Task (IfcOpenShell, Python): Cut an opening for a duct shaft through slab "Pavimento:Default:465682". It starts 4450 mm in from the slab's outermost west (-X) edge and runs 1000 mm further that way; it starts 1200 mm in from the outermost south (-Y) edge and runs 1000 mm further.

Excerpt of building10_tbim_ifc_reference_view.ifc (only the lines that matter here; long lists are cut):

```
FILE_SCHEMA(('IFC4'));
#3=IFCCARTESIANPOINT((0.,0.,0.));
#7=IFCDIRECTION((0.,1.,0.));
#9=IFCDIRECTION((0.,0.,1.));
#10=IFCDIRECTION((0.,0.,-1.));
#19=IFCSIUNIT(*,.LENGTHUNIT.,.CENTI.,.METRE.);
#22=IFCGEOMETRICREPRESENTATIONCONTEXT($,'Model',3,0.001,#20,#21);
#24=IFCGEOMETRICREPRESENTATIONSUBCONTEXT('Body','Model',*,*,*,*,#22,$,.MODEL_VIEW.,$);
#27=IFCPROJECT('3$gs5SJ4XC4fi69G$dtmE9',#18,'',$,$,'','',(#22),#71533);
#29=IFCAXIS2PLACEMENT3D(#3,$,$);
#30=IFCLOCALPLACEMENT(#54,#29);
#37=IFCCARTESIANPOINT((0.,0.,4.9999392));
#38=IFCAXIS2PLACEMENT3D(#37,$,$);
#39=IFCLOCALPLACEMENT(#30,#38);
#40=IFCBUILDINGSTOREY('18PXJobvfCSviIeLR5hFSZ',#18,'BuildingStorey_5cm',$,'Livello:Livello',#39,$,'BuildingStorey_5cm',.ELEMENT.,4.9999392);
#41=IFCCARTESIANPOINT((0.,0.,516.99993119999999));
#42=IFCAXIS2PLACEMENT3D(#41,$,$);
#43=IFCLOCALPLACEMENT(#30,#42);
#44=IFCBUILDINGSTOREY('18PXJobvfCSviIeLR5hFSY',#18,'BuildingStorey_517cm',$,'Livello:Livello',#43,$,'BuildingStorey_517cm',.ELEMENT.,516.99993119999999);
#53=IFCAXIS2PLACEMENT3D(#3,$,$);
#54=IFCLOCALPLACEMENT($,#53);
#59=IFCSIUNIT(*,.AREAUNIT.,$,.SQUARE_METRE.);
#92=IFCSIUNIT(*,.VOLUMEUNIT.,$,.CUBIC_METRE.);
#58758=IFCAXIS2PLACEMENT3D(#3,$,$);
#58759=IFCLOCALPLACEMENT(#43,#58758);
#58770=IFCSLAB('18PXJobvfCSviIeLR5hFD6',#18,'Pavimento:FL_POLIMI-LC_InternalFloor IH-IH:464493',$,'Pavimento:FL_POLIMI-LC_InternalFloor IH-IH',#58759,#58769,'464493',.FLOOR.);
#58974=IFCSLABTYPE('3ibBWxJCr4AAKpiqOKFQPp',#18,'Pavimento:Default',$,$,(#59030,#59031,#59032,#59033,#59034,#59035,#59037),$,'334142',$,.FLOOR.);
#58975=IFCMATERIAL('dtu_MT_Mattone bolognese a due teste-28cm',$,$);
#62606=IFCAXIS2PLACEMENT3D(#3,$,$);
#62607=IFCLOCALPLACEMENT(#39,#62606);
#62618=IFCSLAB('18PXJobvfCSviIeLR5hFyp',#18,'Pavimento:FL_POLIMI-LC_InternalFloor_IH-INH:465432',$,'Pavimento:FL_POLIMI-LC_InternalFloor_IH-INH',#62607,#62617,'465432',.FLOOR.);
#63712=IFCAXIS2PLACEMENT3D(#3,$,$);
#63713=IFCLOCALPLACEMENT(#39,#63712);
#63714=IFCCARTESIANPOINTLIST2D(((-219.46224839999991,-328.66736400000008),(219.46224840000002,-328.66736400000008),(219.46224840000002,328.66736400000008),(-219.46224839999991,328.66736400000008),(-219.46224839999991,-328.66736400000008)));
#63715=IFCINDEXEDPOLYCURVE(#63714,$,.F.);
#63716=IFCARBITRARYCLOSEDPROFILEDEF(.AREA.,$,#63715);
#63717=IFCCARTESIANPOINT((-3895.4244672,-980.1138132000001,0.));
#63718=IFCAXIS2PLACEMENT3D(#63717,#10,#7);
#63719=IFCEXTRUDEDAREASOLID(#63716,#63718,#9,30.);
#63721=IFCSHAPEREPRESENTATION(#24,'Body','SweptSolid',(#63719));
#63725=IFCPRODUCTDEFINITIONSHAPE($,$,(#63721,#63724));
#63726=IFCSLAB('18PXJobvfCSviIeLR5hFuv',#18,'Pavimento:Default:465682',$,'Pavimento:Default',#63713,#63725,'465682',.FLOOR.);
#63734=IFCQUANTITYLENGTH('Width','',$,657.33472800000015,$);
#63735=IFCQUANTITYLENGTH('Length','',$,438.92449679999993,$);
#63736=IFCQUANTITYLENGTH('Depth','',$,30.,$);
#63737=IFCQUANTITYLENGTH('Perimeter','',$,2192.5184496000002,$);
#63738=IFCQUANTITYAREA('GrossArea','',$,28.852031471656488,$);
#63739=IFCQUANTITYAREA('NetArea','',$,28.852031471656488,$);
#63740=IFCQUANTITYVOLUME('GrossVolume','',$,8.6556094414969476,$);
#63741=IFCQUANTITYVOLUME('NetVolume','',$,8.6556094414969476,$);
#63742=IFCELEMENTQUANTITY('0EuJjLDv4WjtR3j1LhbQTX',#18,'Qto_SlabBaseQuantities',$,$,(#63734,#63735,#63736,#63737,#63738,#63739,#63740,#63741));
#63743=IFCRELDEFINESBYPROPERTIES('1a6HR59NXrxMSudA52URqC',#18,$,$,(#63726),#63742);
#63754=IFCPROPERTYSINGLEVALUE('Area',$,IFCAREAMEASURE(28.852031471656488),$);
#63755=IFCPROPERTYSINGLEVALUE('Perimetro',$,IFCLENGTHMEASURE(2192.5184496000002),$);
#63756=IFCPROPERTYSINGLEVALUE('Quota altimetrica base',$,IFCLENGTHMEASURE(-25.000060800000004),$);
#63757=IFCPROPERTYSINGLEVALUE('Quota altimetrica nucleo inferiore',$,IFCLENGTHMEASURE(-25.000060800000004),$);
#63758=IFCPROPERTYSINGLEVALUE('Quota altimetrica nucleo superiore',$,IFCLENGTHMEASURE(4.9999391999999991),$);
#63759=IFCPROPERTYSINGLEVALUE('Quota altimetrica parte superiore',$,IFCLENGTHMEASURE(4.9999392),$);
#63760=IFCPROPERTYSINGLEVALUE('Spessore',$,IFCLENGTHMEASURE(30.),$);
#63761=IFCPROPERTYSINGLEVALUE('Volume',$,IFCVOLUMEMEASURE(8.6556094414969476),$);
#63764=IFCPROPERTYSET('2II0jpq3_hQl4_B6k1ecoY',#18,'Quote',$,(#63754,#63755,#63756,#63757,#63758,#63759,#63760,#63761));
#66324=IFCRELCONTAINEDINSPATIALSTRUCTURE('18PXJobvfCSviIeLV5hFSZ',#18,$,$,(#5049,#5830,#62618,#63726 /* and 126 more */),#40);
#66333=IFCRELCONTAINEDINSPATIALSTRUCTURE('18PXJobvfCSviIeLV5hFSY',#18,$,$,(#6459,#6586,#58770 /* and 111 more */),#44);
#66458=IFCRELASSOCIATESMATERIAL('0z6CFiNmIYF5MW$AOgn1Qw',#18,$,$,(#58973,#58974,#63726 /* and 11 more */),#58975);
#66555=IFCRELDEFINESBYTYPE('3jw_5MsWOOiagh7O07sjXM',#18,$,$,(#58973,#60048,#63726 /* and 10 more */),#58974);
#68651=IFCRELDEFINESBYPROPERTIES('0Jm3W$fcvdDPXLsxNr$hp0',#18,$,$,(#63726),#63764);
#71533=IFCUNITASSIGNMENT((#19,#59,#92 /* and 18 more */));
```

```python
import numpy as np
import ifcopenshell
import ifcopenshell.api.feature
import ifcopenshell.api.geometry
import ifcopenshell.api.pset
import ifcopenshell.api.root
import ifcopenshell.geom
import ifcopenshell.util.element
import ifcopenshell.util.placement
import ifcopenshell.util.representation
import ifcopenshell.util.shape
import ifcopenshell.util.unit

model = ifcopenshell.open("building10_tbim_ifc_reference_view.ifc")
unit_scale = ifcopenshell.util.unit.calculate_unit_scale(model)
area_scale = ifcopenshell.util.unit.calculate_unit_scale(model, "AREAUNIT")
volume_scale = ifcopenshell.util.unit.calculate_unit_scale(model, "VOLUMEUNIT")
settings = ifcopenshell.geom.settings()


def volume(element):
    """Net volume in cubic metres, openings subtracted."""
    shape = ifcopenshell.geom.create_shape(settings, element)
    return ifcopenshell.util.shape.get_volume(shape.geometry)


slab = model.by_guid("18PXJobvfCSviIeLR5hFuv")
before = volume(slab)

# Extent in the slab's own axes, in metres. The edges named are its -X and -Y sides.
slab_shape = ifcopenshell.geom.create_shape(settings, slab)
vertices = ifcopenshell.util.shape.get_vertices(slab_shape.geometry)
x_min, y_min, bottom = vertices.min(axis=0)
top = vertices[:, 2].max()

opening = ifcopenshell.api.root.create_entity(model, ifc_class="IfcOpeningElement", name="Duct shaft opening", predefined_type="OPENING")
context = ifcopenshell.util.representation.get_context(model, "Model", "Body", "MODEL_VIEW")
width, depth = 1, 1
outline = [(0.0, 0.0), (width, 0.0), (width, depth), (0.0, depth), (0.0, 0.0)]
# Overshoot both faces by 50 mm so the cut is clean.
shape = ifcopenshell.api.geometry.add_slab_representation(
    model, context=context, depth=top - bottom + 0.1, polyline=outline
)
ifcopenshell.api.geometry.assign_representation(model, product=opening, representation=shape)

matrix = ifcopenshell.util.placement.get_local_placement(slab.ObjectPlacement)
matrix[:, 3] = matrix @ np.append(np.array([x_min + 4.45, y_min + 1.2, bottom - 0.05]) / unit_scale, 1.0)
ifcopenshell.api.geometry.edit_object_placement(model, product=opening, matrix=matrix, is_si=False)
ifcopenshell.api.feature.add_feature(model, feature=opening, element=slab)

after = volume(slab)

# Update the slab's stored quantities.
qto = model.by_id(ifcopenshell.util.element.get_pset(slab, "Qto_SlabBaseQuantities", should_inherit=False)["id"])
ifcopenshell.api.pset.edit_qto(model, qto=qto, properties={
    "NetArea": after / (top - bottom) / area_scale,
    "NetVolume": after / volume_scale,
})
pset = model.by_id(ifcopenshell.util.element.get_pset(slab, "Quote", should_inherit=False)["id"])
ifcopenshell.api.pset.edit_pset(model, pset=pset, properties={
    "Area": model.create_entity("IfcAreaMeasure", after / (top - bottom) / area_scale),
    "Volume": model.create_entity("IfcVolumeMeasure", after / volume_scale),
})

print(f"slab volume {before:.3f} -> {after:.3f} m3")

model.write("building10_tbim_ifc_reference_view_rev.ifc")
```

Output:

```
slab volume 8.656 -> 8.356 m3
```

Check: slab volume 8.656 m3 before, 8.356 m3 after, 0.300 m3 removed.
